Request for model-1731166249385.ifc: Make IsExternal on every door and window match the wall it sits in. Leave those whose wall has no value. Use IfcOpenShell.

First a look at what the model holds.

```python
import ifcopenshell
import ifcopenshell.util.element

model = ifcopenshell.open("model-1731166249385.ifc")
print(model.schema)
seen = {}
for e in model.by_type("IfcDoor") + model.by_type("IfcWindow"):
    if not e.FillsVoids:
        continue
    host = e.FillsVoids[0].RelatingOpeningElement.VoidsElements[0].RelatingBuildingElement
    own = ifcopenshell.util.element.get_pset(e, f"Pset_{e.is_a()[3:].removesuffix('StandardCase')}Common", "IsExternal")
    wall = ifcopenshell.util.element.get_pset(host, "Pset_WallCommon", "IsExternal")
    seen[e.is_a(), own, wall] = seen.get((e.is_a(), own, wall), 0) + 1
for (cls, own, wall), count in sorted(seen.items(), key=str):
    print(count, cls, "IsExternal:", own, "| host wall:", wall)
```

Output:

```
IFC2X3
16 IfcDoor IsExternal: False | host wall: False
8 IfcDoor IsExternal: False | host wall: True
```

```python
import ifcopenshell
import ifcopenshell.api.pset
import ifcopenshell.util.element

model = ifcopenshell.open("model-1731166249385.ifc")

count = 0
for ifc_class, pset_name in (("IfcDoor", "Pset_DoorCommon"), ("IfcWindow", "Pset_WindowCommon")):
    for e in model.by_type(ifc_class):
        if not e.FillsVoids:
            continue
        host = e.FillsVoids[0].RelatingOpeningElement.VoidsElements[0].RelatingBuildingElement
        external = ifcopenshell.util.element.get_pset(host, "Pset_WallCommon", "IsExternal")
        if external is None or ifcopenshell.util.element.get_pset(e, pset_name, "IsExternal") == external:
            continue
        pset = ifcopenshell.api.pset.add_pset(model, product=e, name=pset_name)
        ifcopenshell.api.pset.edit_pset(model, pset=pset, properties={"IsExternal": external})
        count += 1

print(count, "updated")

model.write("model-1731166249385-out.ifc")
```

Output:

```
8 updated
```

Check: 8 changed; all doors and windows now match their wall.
